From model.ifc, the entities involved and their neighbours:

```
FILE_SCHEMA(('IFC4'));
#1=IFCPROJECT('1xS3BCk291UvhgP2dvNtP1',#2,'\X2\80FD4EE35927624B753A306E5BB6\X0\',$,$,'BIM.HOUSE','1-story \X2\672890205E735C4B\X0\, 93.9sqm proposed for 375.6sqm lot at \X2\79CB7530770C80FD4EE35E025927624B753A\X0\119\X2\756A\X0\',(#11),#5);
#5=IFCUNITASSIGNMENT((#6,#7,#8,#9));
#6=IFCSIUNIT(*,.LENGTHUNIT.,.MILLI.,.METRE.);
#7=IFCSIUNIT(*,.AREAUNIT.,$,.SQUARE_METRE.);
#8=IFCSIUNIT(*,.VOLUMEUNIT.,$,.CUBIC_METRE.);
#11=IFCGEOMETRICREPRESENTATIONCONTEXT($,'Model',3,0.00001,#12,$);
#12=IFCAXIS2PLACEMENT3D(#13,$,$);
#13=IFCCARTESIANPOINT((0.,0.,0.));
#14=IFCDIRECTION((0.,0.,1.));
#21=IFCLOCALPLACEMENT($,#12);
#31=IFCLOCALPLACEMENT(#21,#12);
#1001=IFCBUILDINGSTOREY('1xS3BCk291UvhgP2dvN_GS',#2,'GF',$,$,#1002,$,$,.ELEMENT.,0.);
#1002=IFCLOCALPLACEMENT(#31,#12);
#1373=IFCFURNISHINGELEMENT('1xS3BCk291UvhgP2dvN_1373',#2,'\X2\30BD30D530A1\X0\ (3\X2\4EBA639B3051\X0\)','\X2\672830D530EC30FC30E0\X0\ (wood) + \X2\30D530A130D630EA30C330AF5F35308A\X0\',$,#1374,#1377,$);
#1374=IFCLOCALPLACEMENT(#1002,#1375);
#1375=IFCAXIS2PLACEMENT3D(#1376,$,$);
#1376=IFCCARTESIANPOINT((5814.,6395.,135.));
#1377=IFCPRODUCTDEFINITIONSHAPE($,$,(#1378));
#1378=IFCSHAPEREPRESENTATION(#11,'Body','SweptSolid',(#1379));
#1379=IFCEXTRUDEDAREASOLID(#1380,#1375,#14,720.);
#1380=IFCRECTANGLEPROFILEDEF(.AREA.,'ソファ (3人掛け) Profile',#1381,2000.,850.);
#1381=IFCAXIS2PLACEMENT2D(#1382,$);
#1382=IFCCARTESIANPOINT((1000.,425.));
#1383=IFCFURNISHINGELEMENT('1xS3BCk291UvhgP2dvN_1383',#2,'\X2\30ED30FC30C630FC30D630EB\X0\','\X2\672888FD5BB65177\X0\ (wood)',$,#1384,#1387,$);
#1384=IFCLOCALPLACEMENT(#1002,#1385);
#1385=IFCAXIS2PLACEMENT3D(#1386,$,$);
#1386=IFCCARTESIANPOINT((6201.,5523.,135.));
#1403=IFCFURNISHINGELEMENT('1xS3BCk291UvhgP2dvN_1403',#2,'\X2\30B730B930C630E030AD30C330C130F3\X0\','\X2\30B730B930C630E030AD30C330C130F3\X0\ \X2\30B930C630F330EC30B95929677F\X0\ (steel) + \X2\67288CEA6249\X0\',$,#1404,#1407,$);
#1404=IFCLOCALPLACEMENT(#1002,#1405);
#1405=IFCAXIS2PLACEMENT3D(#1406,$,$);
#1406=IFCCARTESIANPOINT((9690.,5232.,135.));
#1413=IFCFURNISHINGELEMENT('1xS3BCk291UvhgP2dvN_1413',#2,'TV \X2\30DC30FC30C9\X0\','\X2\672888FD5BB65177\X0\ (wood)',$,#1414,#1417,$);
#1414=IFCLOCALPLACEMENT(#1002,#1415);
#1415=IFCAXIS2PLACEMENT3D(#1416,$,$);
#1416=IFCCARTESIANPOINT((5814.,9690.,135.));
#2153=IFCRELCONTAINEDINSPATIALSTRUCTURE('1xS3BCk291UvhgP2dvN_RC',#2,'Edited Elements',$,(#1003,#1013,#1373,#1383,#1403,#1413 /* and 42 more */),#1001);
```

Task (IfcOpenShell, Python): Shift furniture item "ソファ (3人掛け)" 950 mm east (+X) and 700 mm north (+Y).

```python
import ifcopenshell
import ifcopenshell.api.geometry
import ifcopenshell.util.placement
import ifcopenshell.util.unit

model = ifcopenshell.open("model.ifc")
unit_scale = ifcopenshell.util.unit.calculate_unit_scale(model)

item = model.by_guid("1xS3BCk291UvhgP2dvN_1373")
matrix = ifcopenshell.util.placement.get_local_placement(item.ObjectPlacement)
matrix[0, 3] += 0.95 / unit_scale
matrix[1, 3] += 0.7 / unit_scale
ifcopenshell.api.geometry.edit_object_placement(model, product=item, matrix=matrix, is_si=False)

print(ifcopenshell.util.placement.get_local_placement(item.ObjectPlacement).round(3) + 0.0)

model.write("model_edited.ifc")
```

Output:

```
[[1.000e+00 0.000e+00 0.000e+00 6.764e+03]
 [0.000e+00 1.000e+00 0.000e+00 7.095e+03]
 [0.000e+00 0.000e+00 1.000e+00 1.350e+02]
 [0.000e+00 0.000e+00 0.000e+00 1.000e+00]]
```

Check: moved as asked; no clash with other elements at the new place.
